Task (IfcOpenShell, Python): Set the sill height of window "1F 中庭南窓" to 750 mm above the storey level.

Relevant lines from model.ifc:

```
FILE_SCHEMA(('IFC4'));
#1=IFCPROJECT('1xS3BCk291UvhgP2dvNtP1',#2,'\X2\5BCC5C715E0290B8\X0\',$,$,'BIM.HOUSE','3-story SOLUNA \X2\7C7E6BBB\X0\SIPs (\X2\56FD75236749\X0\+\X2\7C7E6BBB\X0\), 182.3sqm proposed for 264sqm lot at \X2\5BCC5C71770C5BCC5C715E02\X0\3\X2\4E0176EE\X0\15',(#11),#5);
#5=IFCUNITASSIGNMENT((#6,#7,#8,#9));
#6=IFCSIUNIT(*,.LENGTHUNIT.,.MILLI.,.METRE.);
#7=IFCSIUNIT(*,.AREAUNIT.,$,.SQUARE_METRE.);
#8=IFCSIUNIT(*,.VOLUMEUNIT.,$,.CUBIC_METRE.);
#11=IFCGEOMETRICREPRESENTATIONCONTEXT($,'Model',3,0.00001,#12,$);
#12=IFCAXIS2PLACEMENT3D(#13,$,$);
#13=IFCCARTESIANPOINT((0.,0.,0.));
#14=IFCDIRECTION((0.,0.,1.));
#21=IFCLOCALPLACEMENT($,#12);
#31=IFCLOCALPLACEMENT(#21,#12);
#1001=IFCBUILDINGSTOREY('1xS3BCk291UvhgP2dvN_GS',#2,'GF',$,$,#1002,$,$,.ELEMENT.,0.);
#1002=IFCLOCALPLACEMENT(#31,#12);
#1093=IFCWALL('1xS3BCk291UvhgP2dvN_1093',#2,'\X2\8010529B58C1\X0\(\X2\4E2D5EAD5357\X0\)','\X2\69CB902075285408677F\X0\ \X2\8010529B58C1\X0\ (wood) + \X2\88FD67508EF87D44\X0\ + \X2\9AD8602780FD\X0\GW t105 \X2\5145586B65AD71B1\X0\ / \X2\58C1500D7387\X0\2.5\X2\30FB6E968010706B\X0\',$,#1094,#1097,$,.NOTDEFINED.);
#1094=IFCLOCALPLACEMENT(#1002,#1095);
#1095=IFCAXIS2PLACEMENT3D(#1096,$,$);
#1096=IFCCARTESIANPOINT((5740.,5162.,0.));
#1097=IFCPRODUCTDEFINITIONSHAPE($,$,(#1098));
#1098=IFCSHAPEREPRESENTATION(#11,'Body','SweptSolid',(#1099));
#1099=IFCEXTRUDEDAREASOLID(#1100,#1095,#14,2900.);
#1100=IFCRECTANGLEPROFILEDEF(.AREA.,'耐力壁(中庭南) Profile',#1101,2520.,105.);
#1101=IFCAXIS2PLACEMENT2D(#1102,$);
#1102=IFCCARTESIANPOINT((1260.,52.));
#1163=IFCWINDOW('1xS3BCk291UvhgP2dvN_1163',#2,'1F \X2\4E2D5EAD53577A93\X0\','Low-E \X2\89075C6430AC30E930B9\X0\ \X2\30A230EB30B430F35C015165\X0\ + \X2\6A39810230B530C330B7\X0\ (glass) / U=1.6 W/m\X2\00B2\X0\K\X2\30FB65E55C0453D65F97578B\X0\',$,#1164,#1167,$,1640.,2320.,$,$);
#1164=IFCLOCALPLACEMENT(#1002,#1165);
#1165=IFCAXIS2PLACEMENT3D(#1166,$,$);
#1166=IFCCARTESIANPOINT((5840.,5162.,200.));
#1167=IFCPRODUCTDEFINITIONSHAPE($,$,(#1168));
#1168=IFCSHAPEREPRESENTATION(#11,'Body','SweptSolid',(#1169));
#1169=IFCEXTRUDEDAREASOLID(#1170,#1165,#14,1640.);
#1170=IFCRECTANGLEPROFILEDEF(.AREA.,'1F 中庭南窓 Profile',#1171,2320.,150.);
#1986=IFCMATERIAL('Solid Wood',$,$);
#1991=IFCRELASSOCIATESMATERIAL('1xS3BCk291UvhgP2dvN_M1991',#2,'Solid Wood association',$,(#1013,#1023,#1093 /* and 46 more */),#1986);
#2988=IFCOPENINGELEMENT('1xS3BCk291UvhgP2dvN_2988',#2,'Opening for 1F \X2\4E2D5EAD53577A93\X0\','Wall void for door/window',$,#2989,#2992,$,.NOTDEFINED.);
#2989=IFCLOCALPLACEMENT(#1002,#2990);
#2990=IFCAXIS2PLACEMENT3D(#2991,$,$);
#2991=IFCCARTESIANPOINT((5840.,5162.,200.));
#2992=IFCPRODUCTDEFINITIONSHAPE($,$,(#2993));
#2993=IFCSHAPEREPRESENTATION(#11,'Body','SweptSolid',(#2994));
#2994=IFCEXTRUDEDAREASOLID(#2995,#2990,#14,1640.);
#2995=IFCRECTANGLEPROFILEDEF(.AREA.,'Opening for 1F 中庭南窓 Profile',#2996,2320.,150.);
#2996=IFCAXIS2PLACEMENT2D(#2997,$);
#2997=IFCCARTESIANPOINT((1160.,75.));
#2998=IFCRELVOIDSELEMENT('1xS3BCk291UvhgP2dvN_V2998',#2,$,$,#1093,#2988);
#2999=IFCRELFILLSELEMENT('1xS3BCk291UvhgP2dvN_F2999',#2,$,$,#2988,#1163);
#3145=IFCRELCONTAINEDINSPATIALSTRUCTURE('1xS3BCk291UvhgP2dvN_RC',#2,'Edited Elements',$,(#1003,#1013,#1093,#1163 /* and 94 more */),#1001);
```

```python
import numpy as np
import ifcopenshell
import ifcopenshell.api.geometry
import ifcopenshell.geom
import ifcopenshell.util.element
import ifcopenshell.util.placement
import ifcopenshell.util.shape
import ifcopenshell.util.unit

model = ifcopenshell.open("model.ifc")
unit_scale = ifcopenshell.util.unit.calculate_unit_scale(model)

window = model.by_guid("1xS3BCk291UvhgP2dvN_1163")
opening = window.FillsVoids[0].RelatingOpeningElement
storey = ifcopenshell.util.element.get_container(window, ifc_class="IfcBuildingStorey")
level = ifcopenshell.util.placement.get_local_placement(storey.ObjectPlacement)[2, 3]

# The opening's origin need not be at the sill, so measure its lowest point.
shape = ifcopenshell.geom.create_shape(ifcopenshell.geom.settings(), opening)
bottom = ifcopenshell.util.shape.get_shape_bottom_elevation(shape, shape.geometry) / unit_scale
dz = level + 750.0 - bottom

shift = np.array([0.0, 0.0, dz])
# The window is not placed relative to its opening, so move both.
for product in (opening, window):
    matrix = ifcopenshell.util.placement.get_local_placement(product.ObjectPlacement)
    matrix[:3, 3] += shift
    ifcopenshell.api.geometry.edit_object_placement(model, product=product, matrix=matrix, is_si=False)

print(f"moved by {dz * unit_scale:+.3f} m")

model.write("model_v2.ifc")
```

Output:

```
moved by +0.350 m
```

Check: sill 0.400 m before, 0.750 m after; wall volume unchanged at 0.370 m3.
